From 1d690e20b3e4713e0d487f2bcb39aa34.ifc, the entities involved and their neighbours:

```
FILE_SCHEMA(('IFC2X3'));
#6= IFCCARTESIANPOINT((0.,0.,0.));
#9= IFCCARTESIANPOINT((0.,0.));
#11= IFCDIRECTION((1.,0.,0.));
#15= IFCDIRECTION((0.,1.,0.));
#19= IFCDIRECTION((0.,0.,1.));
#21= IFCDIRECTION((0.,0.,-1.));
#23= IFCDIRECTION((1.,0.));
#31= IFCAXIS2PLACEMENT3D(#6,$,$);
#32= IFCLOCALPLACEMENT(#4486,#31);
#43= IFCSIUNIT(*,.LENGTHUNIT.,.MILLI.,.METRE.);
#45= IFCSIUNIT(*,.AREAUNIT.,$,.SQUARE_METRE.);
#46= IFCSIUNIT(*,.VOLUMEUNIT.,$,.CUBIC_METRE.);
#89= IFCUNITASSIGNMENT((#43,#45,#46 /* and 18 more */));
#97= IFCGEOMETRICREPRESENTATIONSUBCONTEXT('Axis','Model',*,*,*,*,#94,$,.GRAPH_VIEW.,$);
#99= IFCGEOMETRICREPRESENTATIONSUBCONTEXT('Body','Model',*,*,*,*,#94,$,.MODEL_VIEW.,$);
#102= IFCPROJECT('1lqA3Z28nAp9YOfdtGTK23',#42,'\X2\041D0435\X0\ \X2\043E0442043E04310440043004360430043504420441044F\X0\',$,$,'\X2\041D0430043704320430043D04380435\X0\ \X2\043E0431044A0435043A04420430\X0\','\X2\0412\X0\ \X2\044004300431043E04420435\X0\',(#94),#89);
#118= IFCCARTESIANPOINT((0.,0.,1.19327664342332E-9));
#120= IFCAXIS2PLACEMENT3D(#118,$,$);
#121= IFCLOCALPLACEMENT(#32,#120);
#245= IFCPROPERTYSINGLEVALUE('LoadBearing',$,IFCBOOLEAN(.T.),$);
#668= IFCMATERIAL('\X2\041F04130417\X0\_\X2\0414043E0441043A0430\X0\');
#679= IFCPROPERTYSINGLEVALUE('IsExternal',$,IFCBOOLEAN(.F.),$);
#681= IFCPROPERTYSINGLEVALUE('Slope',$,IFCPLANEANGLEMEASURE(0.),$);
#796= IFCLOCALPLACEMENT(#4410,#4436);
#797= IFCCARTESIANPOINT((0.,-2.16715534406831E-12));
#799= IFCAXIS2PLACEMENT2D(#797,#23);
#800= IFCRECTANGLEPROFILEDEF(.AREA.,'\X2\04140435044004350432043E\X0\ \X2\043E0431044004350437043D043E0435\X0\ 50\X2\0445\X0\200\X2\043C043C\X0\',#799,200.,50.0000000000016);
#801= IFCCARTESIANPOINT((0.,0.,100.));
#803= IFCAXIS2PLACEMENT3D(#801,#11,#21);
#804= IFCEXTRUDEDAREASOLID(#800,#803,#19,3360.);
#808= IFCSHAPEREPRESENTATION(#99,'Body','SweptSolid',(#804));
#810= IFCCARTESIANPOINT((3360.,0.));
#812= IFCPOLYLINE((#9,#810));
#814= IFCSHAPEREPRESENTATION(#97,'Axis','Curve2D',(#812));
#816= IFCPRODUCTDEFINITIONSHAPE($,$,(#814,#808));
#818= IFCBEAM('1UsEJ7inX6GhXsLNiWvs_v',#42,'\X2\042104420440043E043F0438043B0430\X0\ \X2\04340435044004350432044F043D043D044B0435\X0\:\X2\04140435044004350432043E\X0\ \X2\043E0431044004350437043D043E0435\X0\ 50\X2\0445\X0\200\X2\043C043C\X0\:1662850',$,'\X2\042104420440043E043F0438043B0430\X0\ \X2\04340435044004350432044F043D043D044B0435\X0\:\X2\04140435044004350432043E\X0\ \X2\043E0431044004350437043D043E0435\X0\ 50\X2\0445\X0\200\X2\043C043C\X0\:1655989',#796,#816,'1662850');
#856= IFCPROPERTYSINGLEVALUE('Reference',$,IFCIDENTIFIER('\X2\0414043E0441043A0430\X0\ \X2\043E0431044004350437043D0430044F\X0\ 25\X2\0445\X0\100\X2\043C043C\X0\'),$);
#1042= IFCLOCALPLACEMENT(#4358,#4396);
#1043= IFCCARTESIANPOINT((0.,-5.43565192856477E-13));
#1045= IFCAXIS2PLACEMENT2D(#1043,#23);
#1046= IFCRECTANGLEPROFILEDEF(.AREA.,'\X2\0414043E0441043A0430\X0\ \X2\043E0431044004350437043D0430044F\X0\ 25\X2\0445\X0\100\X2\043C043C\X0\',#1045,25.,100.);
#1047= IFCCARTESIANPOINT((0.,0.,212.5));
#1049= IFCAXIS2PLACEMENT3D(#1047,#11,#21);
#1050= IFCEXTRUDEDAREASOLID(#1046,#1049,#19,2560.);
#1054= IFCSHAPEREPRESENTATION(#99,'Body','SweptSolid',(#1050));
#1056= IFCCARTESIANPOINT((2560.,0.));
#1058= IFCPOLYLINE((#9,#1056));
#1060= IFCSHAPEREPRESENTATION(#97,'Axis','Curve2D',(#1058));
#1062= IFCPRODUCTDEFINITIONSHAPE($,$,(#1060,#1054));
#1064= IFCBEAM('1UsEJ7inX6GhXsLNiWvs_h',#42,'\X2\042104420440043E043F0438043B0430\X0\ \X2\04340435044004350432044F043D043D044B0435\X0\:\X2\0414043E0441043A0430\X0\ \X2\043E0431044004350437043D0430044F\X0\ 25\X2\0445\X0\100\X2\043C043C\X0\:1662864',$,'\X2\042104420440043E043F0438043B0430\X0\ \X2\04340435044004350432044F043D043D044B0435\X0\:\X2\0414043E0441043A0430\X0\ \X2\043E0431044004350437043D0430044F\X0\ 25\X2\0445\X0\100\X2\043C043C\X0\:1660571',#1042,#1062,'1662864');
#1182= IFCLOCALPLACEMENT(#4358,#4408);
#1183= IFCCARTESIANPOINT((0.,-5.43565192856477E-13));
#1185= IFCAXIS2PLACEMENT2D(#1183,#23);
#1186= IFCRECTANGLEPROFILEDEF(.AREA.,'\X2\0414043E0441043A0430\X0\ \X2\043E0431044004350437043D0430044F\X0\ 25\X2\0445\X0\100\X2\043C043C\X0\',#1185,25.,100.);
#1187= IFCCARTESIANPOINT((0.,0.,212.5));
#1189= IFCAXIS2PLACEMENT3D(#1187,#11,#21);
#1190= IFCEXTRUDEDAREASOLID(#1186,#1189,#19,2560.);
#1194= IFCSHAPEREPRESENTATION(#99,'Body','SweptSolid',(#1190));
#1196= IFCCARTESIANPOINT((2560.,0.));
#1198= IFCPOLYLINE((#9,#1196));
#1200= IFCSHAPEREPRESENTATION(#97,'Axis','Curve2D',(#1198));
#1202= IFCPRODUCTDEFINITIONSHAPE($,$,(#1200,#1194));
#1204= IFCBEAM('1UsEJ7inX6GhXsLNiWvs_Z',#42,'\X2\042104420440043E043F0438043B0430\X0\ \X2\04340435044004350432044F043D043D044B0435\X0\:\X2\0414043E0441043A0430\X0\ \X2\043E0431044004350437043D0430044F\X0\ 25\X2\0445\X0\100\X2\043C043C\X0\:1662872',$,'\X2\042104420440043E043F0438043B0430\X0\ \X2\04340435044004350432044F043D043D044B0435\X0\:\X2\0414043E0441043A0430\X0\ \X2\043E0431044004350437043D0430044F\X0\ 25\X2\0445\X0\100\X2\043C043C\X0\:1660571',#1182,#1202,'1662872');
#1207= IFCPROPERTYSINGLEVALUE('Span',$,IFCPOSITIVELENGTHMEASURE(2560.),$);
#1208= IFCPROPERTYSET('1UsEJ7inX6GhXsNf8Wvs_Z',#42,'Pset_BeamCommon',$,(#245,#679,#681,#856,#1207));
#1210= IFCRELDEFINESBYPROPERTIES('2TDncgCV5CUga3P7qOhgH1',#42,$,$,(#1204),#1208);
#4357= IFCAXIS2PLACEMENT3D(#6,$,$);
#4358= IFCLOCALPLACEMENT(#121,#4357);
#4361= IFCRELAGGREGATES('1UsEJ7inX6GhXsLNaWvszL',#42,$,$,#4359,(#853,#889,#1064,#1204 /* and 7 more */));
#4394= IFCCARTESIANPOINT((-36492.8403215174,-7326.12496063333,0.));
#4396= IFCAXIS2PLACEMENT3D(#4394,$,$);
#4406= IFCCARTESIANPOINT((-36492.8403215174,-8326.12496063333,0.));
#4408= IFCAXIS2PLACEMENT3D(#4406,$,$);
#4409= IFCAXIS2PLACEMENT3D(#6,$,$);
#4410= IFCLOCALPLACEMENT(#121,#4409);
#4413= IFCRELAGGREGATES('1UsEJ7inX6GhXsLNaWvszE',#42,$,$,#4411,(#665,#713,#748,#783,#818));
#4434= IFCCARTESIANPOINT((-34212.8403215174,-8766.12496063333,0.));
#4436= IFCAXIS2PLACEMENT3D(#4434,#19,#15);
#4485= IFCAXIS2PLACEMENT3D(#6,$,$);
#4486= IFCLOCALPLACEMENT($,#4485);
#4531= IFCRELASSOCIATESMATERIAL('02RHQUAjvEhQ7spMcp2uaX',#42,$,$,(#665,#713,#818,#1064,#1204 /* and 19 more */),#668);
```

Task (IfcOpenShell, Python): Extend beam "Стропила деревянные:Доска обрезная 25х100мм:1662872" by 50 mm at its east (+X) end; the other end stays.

```python
import numpy as np
import ifcopenshell
import ifcopenshell.api.pset
import ifcopenshell.util.element
import ifcopenshell.util.representation
import ifcopenshell.util.unit

model = ifcopenshell.open("1d690e20b3e4713e0d487f2bcb39aa34.ifc")
unit_scale = ifcopenshell.util.unit.calculate_unit_scale(model)

member = model.by_guid("1UsEJ7inX6GhXsLNiWvs_Z")
change = 0.05 / unit_scale

# The extrusion runs towards the end named, so only its depth changes.
body = ifcopenshell.util.representation.get_representation(member, "Model", "Body")
solid = body.Items[0]
old_length = solid.Depth
solid.Depth += change

# Move the axis end point with it.
axis = next(r for r in member.Representation.Representations if r.RepresentationIdentifier == "Axis").Items[0]
start, end = (np.array(p.Coordinates) for p in axis.Points)
end = end + (end - start) / np.linalg.norm(end - start) * change
point = model.createIfcCartesianPoint(end.tolist())
axis.Points = [axis.Points[0], point]

# Update the stored length and volume.
pset = model.by_id(ifcopenshell.util.element.get_pset(member, "Pset_BeamCommon", should_inherit=False)["id"])
ifcopenshell.api.pset.edit_pset(model, pset=pset, properties={
    "Span": model.create_entity("IfcPositiveLengthMeasure", solid.Depth),
})

print(f"length {old_length:g} -> {solid.Depth:g}")

model.write("1d690e20b3e4713e0d487f2bcb39aa34_updated.ifc")
```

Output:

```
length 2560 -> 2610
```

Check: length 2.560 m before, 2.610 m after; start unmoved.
